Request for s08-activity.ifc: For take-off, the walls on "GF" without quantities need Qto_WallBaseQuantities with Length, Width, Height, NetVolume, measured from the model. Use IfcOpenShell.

First a look at what the model holds.

```python
import ifcopenshell
import ifcopenshell.util.element
import ifcopenshell.util.unit

model = ifcopenshell.open("s08-activity.ifc")
print(model.schema)
for unit_type in ("LENGTHUNIT", "AREAUNIT", "VOLUMEUNIT"):
    print(unit_type, ifcopenshell.util.unit.calculate_unit_scale(model, unit_type))
storey = next(s for s in model.by_type("IfcBuildingStorey") if s.Name == "GF")
walls = [e for e in ifcopenshell.util.element.get_decomposition(storey) if e.is_a("IfcWall")]
for e in sorted(walls, key=lambda e: e.id()):
    print(e.id(), e.is_a(), e.Name, list(ifcopenshell.util.element.get_psets(e, qtos_only=True)), sep=" | ")
```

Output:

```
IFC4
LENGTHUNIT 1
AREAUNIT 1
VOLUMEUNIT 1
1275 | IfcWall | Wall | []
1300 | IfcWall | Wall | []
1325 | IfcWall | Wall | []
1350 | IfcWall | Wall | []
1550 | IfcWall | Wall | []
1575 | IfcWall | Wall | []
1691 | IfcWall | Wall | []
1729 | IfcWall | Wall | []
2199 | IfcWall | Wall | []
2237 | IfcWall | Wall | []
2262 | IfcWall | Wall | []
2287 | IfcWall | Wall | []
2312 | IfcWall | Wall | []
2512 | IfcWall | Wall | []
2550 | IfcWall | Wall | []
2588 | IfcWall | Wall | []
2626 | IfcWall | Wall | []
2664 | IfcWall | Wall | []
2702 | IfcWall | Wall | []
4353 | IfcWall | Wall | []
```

```python
import ifcopenshell
import ifcopenshell.api.pset
import ifcopenshell.geom
import ifcopenshell.util.element
import ifcopenshell.util.shape
import ifcopenshell.util.unit

model = ifcopenshell.open("s08-activity.ifc")
unit_scale = ifcopenshell.util.unit.calculate_unit_scale(model)
volume_scale = ifcopenshell.util.unit.calculate_unit_scale(model, "VOLUMEUNIT")
settings = ifcopenshell.geom.settings()

storey = next(s for s in model.by_type("IfcBuildingStorey") if s.Name == "GF")
walls = [e for e in ifcopenshell.util.element.get_decomposition(storey) if e.is_a("IfcWall")]

for e in sorted(walls, key=lambda e: e.id()):
    if ifcopenshell.util.element.get_psets(e, qtos_only=True, should_inherit=False):
        continue
    # Geometry comes back in metres, in the element's own axes.
    shape = ifcopenshell.geom.create_shape(settings, e)
    values = {
        "Length": ifcopenshell.util.shape.get_x(shape.geometry) / unit_scale,
        "Width": ifcopenshell.util.shape.get_y(shape.geometry) / unit_scale,
        "Height": ifcopenshell.util.shape.get_z(shape.geometry) / unit_scale,
        "NetVolume": ifcopenshell.util.shape.get_volume(shape.geometry) / volume_scale,
    }
    qto = ifcopenshell.api.pset.add_qto(model, product=e, name="Qto_WallBaseQuantities")
    ifcopenshell.api.pset.edit_qto(model, qto=qto, properties=values)
    print(e.id(), {k: round(v, 3) for k, v in values.items()})

model.write("s08-activity_edited.ifc")
```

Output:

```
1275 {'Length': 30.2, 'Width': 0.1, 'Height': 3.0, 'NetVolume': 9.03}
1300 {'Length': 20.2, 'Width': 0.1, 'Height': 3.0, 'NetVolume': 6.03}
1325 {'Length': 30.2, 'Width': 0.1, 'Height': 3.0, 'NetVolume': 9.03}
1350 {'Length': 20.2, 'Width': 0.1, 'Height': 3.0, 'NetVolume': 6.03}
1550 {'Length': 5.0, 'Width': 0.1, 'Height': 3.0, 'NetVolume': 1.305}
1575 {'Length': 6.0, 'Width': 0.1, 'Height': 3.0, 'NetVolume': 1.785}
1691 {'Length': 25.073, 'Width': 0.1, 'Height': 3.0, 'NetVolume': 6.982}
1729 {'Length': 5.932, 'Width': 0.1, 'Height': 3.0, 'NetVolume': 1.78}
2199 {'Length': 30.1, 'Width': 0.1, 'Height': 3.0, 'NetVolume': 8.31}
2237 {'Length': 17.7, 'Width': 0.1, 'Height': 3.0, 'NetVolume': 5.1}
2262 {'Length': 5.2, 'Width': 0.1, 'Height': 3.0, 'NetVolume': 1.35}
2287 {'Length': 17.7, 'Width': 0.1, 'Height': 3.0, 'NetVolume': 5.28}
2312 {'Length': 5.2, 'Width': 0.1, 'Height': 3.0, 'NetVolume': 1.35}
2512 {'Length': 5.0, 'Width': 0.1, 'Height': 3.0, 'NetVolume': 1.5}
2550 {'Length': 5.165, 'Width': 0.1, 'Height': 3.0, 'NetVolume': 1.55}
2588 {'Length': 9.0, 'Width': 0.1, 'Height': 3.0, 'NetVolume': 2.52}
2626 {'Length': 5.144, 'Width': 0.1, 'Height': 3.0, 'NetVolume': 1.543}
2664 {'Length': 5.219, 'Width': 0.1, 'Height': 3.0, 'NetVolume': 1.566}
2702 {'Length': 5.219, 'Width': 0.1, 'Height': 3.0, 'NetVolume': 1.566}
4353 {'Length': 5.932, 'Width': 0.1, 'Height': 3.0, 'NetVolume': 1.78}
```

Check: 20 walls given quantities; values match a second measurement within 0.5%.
